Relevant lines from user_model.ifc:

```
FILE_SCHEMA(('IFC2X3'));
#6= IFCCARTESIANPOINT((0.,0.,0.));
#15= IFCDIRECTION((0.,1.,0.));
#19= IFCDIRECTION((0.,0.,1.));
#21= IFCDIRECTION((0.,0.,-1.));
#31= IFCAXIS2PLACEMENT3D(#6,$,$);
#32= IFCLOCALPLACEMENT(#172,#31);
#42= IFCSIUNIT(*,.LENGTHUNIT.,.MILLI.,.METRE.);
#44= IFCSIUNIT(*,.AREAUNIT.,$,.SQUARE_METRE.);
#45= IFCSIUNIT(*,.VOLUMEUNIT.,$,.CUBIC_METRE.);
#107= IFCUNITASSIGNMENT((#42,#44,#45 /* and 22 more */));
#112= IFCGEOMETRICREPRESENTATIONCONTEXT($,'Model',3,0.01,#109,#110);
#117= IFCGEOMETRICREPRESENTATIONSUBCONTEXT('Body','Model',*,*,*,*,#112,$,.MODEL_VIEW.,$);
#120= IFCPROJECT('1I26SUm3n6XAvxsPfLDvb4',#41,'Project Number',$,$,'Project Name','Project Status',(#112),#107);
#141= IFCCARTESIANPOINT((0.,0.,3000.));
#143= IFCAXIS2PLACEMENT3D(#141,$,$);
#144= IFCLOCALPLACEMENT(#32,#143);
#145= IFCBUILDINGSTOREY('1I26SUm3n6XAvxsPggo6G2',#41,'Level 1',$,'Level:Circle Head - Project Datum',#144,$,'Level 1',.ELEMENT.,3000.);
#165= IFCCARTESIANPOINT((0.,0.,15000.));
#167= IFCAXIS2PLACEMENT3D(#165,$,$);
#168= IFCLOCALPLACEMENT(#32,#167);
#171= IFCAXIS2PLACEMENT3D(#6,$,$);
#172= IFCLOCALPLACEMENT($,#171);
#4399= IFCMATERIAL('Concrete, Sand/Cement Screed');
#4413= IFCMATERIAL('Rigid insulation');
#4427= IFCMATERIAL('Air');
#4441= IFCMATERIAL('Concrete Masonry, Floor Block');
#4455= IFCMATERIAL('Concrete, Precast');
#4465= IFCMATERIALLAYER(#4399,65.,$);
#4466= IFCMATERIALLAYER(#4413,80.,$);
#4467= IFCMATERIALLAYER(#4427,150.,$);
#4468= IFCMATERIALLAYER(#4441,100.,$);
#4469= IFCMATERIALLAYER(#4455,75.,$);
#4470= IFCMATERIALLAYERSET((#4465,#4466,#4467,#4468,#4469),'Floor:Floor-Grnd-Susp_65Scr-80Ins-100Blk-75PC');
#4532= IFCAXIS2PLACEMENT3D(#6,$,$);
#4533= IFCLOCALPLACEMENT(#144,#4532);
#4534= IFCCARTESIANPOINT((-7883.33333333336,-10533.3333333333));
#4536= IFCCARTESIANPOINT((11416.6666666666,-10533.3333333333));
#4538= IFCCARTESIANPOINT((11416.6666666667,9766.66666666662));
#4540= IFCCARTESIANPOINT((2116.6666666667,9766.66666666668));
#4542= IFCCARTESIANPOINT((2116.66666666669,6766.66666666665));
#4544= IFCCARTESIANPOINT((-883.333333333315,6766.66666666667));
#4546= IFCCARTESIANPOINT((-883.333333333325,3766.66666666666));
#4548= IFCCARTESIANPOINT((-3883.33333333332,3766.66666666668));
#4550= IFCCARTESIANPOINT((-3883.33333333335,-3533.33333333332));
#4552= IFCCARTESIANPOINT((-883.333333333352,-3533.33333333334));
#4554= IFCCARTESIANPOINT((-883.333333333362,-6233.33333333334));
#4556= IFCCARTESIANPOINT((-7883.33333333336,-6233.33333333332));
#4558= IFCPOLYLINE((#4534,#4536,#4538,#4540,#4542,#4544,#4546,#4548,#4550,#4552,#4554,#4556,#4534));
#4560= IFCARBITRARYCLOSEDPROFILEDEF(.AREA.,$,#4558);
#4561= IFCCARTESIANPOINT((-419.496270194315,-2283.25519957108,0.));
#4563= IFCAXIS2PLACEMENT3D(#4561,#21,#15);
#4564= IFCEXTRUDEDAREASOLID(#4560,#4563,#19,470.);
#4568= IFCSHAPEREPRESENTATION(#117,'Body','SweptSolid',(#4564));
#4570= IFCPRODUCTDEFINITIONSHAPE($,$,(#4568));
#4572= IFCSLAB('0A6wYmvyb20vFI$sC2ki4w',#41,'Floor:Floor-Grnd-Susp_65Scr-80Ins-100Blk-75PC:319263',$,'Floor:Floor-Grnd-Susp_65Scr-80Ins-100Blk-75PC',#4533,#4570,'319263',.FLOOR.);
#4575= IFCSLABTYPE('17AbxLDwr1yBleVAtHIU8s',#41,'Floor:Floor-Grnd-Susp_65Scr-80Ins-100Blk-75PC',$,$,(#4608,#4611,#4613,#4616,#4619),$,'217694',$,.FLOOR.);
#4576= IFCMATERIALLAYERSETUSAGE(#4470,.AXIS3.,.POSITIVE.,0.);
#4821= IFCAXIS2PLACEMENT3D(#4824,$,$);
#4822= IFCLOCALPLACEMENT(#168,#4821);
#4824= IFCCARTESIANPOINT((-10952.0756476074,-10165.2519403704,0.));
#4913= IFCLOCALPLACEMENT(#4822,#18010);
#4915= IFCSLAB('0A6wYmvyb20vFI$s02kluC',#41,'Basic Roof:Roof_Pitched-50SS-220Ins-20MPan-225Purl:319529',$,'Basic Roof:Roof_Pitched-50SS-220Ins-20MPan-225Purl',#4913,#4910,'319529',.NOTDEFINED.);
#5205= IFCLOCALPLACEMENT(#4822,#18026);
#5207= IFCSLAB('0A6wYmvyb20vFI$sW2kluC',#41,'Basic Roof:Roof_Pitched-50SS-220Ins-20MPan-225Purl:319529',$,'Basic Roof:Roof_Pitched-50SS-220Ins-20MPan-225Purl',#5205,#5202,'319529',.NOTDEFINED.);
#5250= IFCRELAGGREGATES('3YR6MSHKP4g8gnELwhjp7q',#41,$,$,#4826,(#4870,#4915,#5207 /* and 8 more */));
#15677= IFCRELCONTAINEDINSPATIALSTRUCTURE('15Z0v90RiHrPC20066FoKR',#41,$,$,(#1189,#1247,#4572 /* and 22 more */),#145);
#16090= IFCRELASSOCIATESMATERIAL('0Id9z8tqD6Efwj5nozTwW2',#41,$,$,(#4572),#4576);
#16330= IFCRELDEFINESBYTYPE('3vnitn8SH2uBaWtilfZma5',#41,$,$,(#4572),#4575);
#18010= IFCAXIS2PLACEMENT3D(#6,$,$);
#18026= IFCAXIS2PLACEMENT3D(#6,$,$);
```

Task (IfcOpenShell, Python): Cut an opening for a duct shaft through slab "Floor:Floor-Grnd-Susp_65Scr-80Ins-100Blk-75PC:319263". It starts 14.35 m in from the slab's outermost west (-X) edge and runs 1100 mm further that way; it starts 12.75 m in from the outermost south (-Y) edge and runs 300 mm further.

```python
import numpy as np
import ifcopenshell
import ifcopenshell.api.feature
import ifcopenshell.api.geometry
import ifcopenshell.api.root
import ifcopenshell.geom
import ifcopenshell.util.placement
import ifcopenshell.util.representation
import ifcopenshell.util.shape
import ifcopenshell.util.unit

model = ifcopenshell.open("user_model.ifc")
unit_scale = ifcopenshell.util.unit.calculate_unit_scale(model)
settings = ifcopenshell.geom.settings()


def volume(element):
    """Net volume in cubic metres, openings subtracted."""
    shape = ifcopenshell.geom.create_shape(settings, element)
    return ifcopenshell.util.shape.get_volume(shape.geometry)


slab = model.by_id(4572)
before = volume(slab)

# Extent in the slab's own axes, in metres. The edges named are its -X and -Y sides.
slab_shape = ifcopenshell.geom.create_shape(settings, slab)
vertices = ifcopenshell.util.shape.get_vertices(slab_shape.geometry)
x_min, y_min, bottom = vertices.min(axis=0)
top = vertices[:, 2].max()

opening = ifcopenshell.api.root.create_entity(model, ifc_class="IfcOpeningElement", name="Duct shaft opening")
context = ifcopenshell.util.representation.get_context(model, "Model", "Body", "MODEL_VIEW")
width, depth = 1.1, 0.3
outline = [(0.0, 0.0), (width, 0.0), (width, depth), (0.0, depth), (0.0, 0.0)]
# Overshoot both faces by 50 mm so the cut is clean.
shape = ifcopenshell.api.geometry.add_slab_representation(
    model, context=context, depth=top - bottom + 0.1, polyline=outline
)
ifcopenshell.api.geometry.assign_representation(model, product=opening, representation=shape)

matrix = ifcopenshell.util.placement.get_local_placement(slab.ObjectPlacement)
matrix[:, 3] = matrix @ np.append(np.array([x_min + 14.35, y_min + 12.75, bottom - 0.05]) / unit_scale, 1.0)
ifcopenshell.api.geometry.edit_object_placement(model, product=opening, matrix=matrix, is_si=False)
ifcopenshell.api.feature.add_feature(model, feature=opening, element=slab)

after = volume(slab)

print(f"slab volume {before:.3f} -> {after:.3f} m3")

model.write("user_model_rev.ifc")
```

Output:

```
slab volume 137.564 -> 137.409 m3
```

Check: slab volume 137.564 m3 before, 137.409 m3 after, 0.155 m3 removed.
